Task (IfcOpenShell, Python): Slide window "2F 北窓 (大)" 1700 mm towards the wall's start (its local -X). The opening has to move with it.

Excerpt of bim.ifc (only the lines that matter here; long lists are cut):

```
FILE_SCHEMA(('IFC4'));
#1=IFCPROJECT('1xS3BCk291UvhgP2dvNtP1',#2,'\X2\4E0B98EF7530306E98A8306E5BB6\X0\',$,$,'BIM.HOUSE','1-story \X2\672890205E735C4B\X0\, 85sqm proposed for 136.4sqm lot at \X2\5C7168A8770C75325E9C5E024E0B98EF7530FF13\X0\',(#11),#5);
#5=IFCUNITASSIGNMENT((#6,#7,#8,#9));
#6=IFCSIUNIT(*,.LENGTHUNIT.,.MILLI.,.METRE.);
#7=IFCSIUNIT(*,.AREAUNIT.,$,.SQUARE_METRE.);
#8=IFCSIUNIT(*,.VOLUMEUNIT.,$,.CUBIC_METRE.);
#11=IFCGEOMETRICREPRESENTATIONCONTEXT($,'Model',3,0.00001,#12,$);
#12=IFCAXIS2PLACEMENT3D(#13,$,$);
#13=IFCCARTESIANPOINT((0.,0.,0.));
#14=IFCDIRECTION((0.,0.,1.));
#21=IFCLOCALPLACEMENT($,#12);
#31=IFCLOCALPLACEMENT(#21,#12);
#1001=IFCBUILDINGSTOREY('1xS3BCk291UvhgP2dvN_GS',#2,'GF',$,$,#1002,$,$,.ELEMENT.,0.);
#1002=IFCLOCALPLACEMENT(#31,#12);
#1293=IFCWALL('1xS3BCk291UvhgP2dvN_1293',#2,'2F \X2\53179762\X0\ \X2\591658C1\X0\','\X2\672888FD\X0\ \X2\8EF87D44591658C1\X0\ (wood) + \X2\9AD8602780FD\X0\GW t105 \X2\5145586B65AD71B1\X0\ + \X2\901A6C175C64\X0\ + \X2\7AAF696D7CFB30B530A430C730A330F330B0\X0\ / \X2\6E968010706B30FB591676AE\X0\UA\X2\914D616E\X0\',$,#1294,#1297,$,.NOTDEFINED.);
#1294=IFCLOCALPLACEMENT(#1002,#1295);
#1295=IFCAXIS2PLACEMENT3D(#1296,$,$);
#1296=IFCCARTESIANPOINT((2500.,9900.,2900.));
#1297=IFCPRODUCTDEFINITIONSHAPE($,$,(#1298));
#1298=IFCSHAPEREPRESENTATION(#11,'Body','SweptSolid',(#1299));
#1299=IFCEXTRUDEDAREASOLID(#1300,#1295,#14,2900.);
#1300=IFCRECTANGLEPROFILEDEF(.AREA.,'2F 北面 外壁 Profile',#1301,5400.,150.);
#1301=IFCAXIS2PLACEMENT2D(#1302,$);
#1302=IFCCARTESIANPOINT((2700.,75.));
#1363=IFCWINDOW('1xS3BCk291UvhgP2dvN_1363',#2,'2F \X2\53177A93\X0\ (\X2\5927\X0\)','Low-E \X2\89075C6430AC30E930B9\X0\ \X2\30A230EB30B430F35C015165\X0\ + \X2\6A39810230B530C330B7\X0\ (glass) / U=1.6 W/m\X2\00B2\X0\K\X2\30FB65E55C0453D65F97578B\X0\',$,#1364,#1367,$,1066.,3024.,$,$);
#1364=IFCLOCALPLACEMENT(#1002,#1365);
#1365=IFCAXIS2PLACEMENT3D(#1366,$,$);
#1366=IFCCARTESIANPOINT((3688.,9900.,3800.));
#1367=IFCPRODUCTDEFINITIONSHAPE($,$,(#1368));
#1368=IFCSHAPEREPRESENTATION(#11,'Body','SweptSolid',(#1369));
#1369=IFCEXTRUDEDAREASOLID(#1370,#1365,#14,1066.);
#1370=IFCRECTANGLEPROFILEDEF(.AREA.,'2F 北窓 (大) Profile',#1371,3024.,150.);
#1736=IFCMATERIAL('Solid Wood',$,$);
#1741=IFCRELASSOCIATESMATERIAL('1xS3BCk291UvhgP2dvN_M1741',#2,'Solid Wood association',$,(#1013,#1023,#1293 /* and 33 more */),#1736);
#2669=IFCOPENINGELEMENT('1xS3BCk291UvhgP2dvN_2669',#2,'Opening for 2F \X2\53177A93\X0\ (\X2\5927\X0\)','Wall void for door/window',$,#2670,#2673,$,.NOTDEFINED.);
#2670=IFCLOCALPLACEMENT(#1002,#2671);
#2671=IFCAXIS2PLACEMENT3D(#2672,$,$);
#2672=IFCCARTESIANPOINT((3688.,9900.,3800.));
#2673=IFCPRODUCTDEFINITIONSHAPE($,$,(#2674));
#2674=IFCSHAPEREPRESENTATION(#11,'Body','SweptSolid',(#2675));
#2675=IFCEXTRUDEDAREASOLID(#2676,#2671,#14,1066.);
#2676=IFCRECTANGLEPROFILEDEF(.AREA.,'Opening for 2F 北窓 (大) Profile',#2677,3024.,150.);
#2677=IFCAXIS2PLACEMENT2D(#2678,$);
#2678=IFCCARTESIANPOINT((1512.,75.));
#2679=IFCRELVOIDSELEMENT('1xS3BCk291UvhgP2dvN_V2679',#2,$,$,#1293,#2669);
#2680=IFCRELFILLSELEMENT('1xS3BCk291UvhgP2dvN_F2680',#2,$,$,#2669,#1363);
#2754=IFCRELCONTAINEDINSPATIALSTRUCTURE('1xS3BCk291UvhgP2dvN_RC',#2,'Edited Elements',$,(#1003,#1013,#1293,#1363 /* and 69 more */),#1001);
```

```python
import ifcopenshell
import ifcopenshell.api.geometry
import ifcopenshell.util.placement
import ifcopenshell.util.unit

model = ifcopenshell.open("bim.ifc")
unit_scale = ifcopenshell.util.unit.calculate_unit_scale(model)

window = model.by_guid("1xS3BCk291UvhgP2dvN_1363")
opening = window.FillsVoids[0].RelatingOpeningElement
wall = opening.VoidsElements[0].RelatingBuildingElement

wall_matrix = ifcopenshell.util.placement.get_local_placement(wall.ObjectPlacement)
shift = wall_matrix[:3, 0] * -1.7 / unit_scale
before = ifcopenshell.util.placement.get_local_placement(window.ObjectPlacement)[:3, 3].copy()

# The window is not placed relative to its opening, so move both.
for product in (opening, window):
    matrix = ifcopenshell.util.placement.get_local_placement(product.ObjectPlacement)
    matrix[:3, 3] += shift
    ifcopenshell.api.geometry.edit_object_placement(model, product=product, matrix=matrix, is_si=False)

after = ifcopenshell.util.placement.get_local_placement(window.ObjectPlacement)[:3, 3]
print("window moved by", (after - before).round(3) + 0.0)

model.write("bim_edited.ifc")
```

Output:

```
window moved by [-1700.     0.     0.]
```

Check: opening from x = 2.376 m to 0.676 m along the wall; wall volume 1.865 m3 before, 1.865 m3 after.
